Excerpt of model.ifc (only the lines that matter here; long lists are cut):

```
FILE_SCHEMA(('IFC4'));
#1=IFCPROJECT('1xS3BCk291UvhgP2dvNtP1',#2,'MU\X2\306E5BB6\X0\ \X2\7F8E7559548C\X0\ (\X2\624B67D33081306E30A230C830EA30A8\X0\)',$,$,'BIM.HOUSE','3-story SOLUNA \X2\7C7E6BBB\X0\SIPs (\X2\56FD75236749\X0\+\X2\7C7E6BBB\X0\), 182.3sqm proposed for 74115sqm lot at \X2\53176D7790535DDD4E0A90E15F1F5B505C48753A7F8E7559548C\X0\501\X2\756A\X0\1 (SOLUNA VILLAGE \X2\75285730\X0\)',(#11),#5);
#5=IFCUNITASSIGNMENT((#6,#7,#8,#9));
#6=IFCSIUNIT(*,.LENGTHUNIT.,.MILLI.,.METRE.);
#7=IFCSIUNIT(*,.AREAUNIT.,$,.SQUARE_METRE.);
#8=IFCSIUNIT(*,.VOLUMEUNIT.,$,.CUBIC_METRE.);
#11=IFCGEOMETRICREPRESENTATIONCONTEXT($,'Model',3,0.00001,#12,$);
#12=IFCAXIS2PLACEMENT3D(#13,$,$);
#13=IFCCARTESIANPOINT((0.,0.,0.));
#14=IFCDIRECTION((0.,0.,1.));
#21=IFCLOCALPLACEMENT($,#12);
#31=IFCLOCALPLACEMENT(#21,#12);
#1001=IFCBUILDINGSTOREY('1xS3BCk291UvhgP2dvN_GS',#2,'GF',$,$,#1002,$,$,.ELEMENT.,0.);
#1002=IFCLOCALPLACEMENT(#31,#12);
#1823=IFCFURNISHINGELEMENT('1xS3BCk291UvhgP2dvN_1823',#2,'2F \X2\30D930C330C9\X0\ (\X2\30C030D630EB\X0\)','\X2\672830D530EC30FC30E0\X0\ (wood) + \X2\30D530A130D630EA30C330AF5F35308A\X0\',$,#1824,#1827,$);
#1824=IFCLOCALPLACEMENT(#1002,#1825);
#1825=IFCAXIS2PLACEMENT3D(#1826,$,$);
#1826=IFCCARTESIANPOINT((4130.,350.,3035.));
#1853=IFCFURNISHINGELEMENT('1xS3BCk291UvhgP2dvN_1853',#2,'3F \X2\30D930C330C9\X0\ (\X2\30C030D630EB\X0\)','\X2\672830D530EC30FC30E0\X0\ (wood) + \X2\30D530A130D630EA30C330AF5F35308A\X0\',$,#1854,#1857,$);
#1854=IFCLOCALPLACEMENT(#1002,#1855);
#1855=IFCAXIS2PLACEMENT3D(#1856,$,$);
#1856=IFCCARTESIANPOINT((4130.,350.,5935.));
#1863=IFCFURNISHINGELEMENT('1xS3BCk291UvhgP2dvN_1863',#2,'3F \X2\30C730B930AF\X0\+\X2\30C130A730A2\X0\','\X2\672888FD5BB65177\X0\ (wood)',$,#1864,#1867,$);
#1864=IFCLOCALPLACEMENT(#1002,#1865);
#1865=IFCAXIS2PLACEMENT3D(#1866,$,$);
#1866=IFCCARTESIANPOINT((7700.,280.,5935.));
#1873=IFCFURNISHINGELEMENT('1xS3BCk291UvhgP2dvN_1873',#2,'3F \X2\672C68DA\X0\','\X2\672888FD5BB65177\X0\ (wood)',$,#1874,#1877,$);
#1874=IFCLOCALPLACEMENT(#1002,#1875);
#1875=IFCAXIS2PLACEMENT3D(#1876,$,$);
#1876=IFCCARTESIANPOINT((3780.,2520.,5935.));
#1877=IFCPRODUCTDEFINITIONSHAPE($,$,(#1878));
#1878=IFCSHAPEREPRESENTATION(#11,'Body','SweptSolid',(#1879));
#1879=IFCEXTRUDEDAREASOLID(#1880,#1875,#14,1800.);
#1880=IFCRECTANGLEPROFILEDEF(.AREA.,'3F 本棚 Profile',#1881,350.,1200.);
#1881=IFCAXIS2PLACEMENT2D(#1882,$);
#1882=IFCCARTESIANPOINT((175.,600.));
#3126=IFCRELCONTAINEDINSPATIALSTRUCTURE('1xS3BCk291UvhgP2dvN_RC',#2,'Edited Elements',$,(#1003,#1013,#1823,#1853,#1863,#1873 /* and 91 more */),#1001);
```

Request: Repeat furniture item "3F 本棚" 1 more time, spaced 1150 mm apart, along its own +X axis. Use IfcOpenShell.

```python
import ifcopenshell
import ifcopenshell.api.geometry
import ifcopenshell.api.root
import ifcopenshell.util.element
import ifcopenshell.util.placement
import ifcopenshell.util.unit

model = ifcopenshell.open("model.ifc")
unit_scale = ifcopenshell.util.unit.calculate_unit_scale(model)


def reuse_history(source, copy):
    """copy_class also copies each property set's owner history, people and application; keep the originals."""
    for rel in copy.IsDefinedBy:
        if rel.is_a("IfcRelDefinesByProperties") and (history := rel.RelatingPropertyDefinition.OwnerHistory):
            rel.RelatingPropertyDefinition.OwnerHistory = source.OwnerHistory
            ifcopenshell.util.element.remove_deep2(model, history)


source = model.by_id(1873)
base = ifcopenshell.util.placement.get_local_placement(source.ObjectPlacement)
step = base[:3, 0] * 1.15 / unit_scale

for i in range(1, 2):
    copy = ifcopenshell.api.root.copy_class(model, product=source)
    copy.Representation = ifcopenshell.util.element.copy_deep(
        model, source.Representation, exclude=["IfcGeometricRepresentationContext", "IfcRepresentationMap"]
    )
    reuse_history(source, copy)
    matrix = base.copy()
    matrix[:3, 3] += i * step
    print("added at", matrix[:3, 3].round(3) + 0.0)
    ifcopenshell.api.geometry.edit_object_placement(model, product=copy, matrix=matrix, is_si=False)

model.write("model_edited.ifc")
```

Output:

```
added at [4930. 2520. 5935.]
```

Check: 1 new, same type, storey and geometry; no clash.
